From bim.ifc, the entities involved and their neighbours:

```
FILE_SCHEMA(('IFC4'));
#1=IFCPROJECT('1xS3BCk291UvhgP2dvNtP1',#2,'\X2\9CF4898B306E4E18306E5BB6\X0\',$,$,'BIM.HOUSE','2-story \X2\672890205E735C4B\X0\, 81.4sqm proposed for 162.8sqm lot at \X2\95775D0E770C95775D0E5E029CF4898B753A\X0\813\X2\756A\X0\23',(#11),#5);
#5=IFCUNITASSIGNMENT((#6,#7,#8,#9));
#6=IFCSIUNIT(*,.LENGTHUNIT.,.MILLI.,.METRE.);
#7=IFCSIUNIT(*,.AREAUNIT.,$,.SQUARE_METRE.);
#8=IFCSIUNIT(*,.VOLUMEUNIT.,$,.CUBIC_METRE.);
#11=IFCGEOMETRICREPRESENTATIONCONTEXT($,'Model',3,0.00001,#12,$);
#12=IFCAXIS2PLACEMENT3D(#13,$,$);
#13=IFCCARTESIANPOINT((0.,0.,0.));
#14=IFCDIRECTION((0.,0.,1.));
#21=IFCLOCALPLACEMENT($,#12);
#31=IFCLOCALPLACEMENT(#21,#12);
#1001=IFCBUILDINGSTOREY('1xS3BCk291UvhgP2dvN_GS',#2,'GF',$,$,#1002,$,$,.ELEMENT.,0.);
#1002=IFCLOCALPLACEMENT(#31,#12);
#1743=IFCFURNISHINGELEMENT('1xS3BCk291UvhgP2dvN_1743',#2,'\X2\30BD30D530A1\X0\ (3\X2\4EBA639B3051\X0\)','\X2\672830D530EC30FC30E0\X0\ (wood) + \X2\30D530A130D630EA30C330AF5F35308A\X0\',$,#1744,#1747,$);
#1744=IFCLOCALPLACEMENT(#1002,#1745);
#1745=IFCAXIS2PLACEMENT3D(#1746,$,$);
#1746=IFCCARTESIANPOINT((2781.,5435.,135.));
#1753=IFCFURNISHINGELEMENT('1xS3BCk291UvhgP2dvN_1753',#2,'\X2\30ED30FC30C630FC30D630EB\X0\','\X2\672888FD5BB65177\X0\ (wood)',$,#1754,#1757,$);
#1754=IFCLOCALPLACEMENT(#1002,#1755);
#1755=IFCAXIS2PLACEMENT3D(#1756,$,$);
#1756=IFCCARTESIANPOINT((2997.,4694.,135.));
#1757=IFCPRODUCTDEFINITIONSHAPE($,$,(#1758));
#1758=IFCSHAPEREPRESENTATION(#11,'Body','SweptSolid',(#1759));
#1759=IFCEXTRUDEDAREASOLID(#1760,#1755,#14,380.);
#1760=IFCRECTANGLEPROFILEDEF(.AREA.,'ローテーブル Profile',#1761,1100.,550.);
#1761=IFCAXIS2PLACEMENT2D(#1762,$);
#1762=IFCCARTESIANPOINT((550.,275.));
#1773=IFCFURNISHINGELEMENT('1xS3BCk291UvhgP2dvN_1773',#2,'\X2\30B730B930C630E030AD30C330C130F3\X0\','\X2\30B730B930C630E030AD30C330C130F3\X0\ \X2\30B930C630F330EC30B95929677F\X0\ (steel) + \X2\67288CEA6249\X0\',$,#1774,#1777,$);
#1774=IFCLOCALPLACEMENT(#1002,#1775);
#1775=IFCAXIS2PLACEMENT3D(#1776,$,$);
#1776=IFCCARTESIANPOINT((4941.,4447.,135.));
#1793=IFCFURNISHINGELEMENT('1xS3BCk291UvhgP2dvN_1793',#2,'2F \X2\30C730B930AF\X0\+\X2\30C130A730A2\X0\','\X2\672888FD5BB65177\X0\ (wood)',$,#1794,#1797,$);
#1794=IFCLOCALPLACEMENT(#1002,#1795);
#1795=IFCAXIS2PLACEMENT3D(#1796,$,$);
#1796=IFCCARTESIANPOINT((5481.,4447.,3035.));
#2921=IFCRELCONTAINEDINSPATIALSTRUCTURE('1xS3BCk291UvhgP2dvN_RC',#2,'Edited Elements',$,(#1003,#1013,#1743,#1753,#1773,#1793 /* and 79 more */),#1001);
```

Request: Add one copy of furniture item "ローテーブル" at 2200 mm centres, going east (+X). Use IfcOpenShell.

```python
import numpy as np
import ifcopenshell
import ifcopenshell.api.geometry
import ifcopenshell.api.root
import ifcopenshell.util.element
import ifcopenshell.util.placement

model = ifcopenshell.open("bim.ifc")


def reuse_history(source, copy):
    """copy_class also copies each property set's owner history, people and application; keep the originals."""
    for rel in copy.IsDefinedBy:
        if rel.is_a("IfcRelDefinesByProperties") and (history := rel.RelatingPropertyDefinition.OwnerHistory):
            rel.RelatingPropertyDefinition.OwnerHistory = source.OwnerHistory
            ifcopenshell.util.element.remove_deep2(model, history)


source = model.by_id(1753)
base = ifcopenshell.util.placement.get_local_placement(source.ObjectPlacement)
step = np.array([1.0, 0.0, 0.0]) * 2200.0

for i in range(1, 2):
    copy = ifcopenshell.api.root.copy_class(model, product=source)
    copy.Representation = ifcopenshell.util.element.copy_deep(
        model, source.Representation, exclude=["IfcGeometricRepresentationContext", "IfcRepresentationMap"]
    )
    reuse_history(source, copy)
    matrix = base.copy()
    matrix[:3, 3] += i * step
    print("added at", matrix[:3, 3].round(3) + 0.0)
    ifcopenshell.api.geometry.edit_object_placement(model, product=copy, matrix=matrix, is_si=False)

model.write("bim_updated.ifc")
```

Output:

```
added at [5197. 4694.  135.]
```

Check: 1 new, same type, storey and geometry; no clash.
